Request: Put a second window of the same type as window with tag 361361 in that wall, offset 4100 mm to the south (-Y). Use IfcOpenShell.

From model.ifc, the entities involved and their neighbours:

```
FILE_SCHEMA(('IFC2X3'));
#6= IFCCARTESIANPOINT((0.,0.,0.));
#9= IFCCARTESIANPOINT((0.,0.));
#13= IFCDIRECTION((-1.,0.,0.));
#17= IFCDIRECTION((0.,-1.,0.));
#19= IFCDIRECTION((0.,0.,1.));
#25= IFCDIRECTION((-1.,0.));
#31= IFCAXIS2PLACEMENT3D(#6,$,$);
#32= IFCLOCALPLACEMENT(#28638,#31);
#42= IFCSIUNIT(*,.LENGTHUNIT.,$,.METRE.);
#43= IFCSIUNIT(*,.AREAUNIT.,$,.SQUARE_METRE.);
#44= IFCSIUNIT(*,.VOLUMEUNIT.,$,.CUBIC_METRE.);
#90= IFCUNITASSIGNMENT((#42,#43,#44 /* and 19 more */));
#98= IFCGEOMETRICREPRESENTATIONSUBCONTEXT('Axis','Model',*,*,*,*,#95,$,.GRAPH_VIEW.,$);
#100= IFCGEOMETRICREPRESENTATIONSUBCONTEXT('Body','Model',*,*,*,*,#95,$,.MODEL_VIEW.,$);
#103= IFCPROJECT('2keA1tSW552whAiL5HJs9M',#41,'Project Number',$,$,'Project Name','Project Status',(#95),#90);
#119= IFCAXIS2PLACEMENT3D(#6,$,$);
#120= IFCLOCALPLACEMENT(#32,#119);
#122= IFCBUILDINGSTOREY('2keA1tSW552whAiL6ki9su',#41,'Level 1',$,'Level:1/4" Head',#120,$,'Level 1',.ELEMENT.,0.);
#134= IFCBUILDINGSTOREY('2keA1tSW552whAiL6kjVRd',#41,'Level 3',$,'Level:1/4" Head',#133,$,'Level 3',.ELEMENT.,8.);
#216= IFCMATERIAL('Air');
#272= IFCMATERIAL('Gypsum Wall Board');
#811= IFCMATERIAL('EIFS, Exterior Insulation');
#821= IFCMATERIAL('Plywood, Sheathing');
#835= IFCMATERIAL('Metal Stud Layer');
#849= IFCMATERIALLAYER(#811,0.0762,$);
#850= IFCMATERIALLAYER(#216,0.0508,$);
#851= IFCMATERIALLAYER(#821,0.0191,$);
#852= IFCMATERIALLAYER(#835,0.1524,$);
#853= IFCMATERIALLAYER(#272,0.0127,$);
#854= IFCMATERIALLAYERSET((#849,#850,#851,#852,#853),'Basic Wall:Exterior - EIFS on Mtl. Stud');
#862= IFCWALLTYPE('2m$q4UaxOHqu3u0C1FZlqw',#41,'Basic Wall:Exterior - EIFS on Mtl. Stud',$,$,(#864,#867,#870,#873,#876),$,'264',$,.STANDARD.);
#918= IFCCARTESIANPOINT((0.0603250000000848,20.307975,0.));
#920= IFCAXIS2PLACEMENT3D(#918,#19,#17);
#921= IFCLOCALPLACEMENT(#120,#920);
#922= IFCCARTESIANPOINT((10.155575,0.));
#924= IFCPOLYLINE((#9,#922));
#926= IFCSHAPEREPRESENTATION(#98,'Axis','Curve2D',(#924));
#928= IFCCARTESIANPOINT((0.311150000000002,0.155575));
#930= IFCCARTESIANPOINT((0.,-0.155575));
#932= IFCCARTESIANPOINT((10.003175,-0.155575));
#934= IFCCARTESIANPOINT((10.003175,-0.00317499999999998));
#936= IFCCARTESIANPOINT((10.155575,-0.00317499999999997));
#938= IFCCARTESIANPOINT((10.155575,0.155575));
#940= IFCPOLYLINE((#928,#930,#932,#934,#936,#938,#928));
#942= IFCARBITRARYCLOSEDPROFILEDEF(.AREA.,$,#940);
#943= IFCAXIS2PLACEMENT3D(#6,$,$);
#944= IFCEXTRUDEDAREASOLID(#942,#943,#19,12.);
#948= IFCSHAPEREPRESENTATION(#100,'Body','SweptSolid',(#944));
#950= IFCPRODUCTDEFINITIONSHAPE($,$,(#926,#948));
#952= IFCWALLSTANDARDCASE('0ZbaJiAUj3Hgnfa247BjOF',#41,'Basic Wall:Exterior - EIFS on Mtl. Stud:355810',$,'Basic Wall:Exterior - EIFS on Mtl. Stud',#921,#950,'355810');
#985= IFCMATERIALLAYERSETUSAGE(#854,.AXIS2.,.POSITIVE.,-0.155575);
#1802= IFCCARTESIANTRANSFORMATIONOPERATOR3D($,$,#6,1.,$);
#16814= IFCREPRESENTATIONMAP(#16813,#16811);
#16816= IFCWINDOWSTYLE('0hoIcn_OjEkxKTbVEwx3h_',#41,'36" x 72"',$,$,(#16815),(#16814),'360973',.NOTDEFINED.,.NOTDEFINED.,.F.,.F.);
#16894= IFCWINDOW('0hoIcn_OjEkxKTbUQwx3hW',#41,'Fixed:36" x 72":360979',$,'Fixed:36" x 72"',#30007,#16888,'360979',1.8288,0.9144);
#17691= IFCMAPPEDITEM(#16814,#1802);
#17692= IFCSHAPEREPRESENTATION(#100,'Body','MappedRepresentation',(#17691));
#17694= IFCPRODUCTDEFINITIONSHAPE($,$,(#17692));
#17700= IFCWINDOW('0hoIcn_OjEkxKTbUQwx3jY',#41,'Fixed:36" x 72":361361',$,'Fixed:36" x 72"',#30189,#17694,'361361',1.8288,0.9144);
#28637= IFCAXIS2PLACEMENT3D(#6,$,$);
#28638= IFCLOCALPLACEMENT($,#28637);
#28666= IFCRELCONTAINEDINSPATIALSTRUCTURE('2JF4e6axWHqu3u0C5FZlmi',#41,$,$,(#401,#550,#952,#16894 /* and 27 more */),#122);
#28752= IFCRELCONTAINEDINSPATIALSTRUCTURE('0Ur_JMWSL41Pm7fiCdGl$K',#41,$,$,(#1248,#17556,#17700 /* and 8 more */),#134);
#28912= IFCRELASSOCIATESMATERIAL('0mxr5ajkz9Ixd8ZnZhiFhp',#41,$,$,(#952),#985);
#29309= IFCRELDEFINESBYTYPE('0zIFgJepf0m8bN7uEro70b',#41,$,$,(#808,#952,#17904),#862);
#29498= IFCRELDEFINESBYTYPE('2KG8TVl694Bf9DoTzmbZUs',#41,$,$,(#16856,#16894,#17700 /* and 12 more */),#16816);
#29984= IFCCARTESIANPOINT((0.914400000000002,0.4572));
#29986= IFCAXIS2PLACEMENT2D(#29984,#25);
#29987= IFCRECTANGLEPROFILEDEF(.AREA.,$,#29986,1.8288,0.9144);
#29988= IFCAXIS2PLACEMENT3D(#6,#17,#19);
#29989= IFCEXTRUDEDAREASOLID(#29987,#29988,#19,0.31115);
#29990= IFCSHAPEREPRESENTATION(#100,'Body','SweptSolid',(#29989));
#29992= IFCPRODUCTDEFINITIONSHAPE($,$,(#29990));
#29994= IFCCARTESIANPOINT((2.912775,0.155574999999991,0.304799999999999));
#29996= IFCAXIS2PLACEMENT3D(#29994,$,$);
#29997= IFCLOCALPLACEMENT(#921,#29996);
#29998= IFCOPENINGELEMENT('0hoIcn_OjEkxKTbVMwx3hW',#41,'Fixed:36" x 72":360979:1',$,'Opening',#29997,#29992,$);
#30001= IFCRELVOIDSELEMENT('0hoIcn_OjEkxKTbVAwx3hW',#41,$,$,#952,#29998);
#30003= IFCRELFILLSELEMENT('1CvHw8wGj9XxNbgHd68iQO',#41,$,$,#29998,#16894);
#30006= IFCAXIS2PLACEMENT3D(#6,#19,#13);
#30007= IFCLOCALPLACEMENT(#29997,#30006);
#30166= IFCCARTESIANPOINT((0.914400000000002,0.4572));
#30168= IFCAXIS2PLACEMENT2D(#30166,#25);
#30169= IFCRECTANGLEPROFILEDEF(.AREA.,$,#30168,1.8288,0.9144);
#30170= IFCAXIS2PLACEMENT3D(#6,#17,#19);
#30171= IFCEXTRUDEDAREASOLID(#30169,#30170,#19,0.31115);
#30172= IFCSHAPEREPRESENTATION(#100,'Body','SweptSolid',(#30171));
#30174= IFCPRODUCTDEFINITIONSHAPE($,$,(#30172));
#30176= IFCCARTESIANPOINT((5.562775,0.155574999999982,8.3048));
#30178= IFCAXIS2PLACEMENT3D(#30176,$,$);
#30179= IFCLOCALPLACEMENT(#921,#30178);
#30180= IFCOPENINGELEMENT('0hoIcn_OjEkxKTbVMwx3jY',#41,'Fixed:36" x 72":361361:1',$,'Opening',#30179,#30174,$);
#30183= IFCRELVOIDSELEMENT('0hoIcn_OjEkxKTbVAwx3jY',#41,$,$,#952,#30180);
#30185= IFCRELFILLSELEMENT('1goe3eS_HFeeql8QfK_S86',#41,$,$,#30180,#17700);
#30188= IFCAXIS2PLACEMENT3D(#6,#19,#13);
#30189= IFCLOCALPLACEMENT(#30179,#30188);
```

```python
import ifcopenshell
import ifcopenshell.api.feature
import ifcopenshell.api.geometry
import ifcopenshell.api.root
import ifcopenshell.geom
import ifcopenshell.util.element
import ifcopenshell.util.placement
import ifcopenshell.util.shape

model = ifcopenshell.open("model.ifc")
settings = ifcopenshell.geom.settings()


def volume(element):
    """Net volume in cubic metres, openings subtracted."""
    shape = ifcopenshell.geom.create_shape(settings, element)
    return ifcopenshell.util.shape.get_volume(shape.geometry)


def reuse_history(source, copy):
    """copy_class also copies each property set's owner history, people and application; keep the originals."""
    for rel in copy.IsDefinedBy:
        if rel.is_a("IfcRelDefinesByProperties") and (history := rel.RelatingPropertyDefinition.OwnerHistory):
            rel.RelatingPropertyDefinition.OwnerHistory = source.OwnerHistory
            ifcopenshell.util.element.remove_deep2(model, history)


window = model.by_guid("0hoIcn_OjEkxKTbUQwx3jY")
opening = window.FillsVoids[0].RelatingOpeningElement
wall = opening.VoidsElements[0].RelatingBuildingElement
before = volume(wall)
shift = ifcopenshell.util.placement.get_local_placement(wall.ObjectPlacement)[:3, 0] * 4.1

# copy_class copies the void relationship, type, container and properties, but no geometry.
new_opening = ifcopenshell.api.root.copy_class(model, product=opening)
new_opening.Representation = ifcopenshell.util.element.copy_deep(
    model, opening.Representation, exclude=["IfcGeometricRepresentationContext", "IfcRepresentationMap"]
)
new_opening.Name = 'Fixed:36" x 72"'
new_window = ifcopenshell.api.root.copy_class(model, product=window)
new_window.Representation = ifcopenshell.util.element.copy_deep(
    model, window.Representation, exclude=["IfcGeometricRepresentationContext", "IfcRepresentationMap"]
)
new_window.Name = 'Fixed:36" x 72"'
new_window.Tag = None
reuse_history(window, new_window)
fills = ifcopenshell.api.feature.add_filling(model, opening=new_opening, element=new_window)
fills.OwnerHistory = new_window.OwnerHistory  # required in IFC2X3

for old, new in ((opening, new_opening), (window, new_window)):
    matrix = ifcopenshell.util.placement.get_local_placement(old.ObjectPlacement)
    matrix[:3, 3] += shift
    ifcopenshell.api.geometry.edit_object_placement(model, product=new, matrix=matrix, is_si=False)

after = volume(wall)

print(f"wall volume {before:.3f} -> {after:.3f} m3")

model.write("model_rev.ifc")
```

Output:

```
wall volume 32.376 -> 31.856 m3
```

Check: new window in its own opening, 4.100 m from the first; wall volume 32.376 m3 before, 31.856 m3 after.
